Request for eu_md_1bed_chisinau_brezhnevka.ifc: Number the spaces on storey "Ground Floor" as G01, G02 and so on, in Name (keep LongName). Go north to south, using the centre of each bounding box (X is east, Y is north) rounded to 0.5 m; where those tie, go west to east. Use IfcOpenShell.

First a look at what the model holds.

```python
import ifcopenshell
import ifcopenshell.util.element
import ifcopenshell.util.placement

model = ifcopenshell.open("eu_md_1bed_chisinau_brezhnevka.ifc")
print(model.schema)
storey = next(s for s in model.by_type("IfcBuildingStorey") if s.Name == "Ground Floor")
spaces = [e for e in ifcopenshell.util.element.get_decomposition(storey) if e.is_a("IfcSpace")]
for e in sorted(spaces, key=lambda e: e.id()):
    origin = ifcopenshell.util.placement.get_local_placement(e.ObjectPlacement)[:3, 3]
    print(e.id(), e.Name, e.LongName, origin.round(2) + 0.0, sep=" | ")
```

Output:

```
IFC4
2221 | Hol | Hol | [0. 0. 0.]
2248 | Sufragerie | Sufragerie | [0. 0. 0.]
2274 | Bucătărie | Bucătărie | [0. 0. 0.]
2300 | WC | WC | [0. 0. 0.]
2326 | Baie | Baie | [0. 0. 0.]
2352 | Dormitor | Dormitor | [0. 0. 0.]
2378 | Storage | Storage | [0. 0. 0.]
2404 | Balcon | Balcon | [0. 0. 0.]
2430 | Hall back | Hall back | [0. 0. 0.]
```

```python
import ifcopenshell
import ifcopenshell.geom
import ifcopenshell.util.element
import ifcopenshell.util.shape

model = ifcopenshell.open("eu_md_1bed_chisinau_brezhnevka.ifc")
settings = ifcopenshell.geom.settings()
settings.set("use-world-coords", True)


def centre(element):
    shape = ifcopenshell.geom.create_shape(settings, element)
    return ifcopenshell.util.shape.get_bbox_centroid(shape.geometry)


storey = next(s for s in model.by_type("IfcBuildingStorey") if s.Name == "Ground Floor")
spaces = [e for e in ifcopenshell.util.element.get_decomposition(storey) if e.is_a("IfcSpace")]

# Insertion points can sit at a corner or the storey origin, so sort by the geometry (in metres).
centres = {e: centre(e) for e in spaces}
spaces.sort(key=lambda e: (-round(centres[e][1] / 0.5), centres[e][0]))

for i, e in enumerate(spaces, start=1):
    number = f"G{i:02d}"
    e.Name = number
    print(e.id(), number)

model.write("eu_md_1bed_chisinau_brezhnevka_updated.ifc")
```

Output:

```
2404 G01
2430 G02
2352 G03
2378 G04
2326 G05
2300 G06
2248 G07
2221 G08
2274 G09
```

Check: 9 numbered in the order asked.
